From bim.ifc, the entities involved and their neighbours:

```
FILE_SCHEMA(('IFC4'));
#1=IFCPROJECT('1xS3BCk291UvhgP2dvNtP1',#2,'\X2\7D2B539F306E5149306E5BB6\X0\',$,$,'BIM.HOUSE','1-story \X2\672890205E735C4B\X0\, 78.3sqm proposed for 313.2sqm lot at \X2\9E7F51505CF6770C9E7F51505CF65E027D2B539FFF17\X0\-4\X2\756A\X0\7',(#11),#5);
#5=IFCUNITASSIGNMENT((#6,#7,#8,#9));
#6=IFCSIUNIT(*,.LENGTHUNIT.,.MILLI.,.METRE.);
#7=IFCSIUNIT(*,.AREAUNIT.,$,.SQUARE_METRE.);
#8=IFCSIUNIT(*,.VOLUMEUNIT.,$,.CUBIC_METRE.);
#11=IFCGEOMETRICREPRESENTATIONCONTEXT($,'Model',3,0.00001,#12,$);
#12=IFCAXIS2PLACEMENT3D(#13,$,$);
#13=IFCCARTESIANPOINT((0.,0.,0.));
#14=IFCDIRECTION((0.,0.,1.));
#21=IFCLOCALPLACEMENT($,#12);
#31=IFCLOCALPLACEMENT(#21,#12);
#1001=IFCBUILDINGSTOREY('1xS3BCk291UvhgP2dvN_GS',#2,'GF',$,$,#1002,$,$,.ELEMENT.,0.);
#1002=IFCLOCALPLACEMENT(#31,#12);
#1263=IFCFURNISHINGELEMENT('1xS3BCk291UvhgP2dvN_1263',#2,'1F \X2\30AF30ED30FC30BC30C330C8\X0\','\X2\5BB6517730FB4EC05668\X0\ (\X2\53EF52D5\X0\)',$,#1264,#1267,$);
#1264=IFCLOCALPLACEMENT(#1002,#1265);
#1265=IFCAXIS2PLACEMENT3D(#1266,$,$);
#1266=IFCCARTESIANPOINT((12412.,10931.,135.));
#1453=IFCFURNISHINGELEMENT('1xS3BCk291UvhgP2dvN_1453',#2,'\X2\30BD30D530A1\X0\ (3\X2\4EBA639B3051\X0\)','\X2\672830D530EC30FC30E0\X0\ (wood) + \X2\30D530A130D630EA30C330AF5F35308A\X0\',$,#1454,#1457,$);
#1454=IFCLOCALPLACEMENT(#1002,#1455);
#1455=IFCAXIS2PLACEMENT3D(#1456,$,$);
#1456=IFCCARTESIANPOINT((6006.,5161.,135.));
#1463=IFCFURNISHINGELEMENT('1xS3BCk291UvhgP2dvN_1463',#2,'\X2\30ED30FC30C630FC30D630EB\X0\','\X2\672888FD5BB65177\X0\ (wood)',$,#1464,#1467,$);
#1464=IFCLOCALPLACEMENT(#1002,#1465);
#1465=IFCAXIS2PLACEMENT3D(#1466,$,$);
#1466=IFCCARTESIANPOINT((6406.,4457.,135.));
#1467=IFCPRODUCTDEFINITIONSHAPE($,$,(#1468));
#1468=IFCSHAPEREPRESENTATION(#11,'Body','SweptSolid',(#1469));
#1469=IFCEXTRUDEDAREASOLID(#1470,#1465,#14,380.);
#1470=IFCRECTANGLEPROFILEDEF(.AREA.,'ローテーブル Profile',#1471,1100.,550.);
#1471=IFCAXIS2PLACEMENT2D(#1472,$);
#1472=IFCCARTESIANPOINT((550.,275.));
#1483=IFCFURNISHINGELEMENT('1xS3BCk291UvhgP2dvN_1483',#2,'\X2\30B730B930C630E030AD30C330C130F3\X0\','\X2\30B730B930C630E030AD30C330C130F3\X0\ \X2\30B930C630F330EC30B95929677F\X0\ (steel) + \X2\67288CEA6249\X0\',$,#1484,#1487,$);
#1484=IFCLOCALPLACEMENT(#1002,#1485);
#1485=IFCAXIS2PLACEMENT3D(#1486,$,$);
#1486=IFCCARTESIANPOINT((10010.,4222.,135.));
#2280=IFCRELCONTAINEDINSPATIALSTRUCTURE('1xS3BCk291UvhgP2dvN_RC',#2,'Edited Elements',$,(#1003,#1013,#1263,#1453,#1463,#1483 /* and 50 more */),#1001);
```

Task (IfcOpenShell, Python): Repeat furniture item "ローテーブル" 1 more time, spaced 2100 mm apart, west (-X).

```python
import numpy as np
import ifcopenshell
import ifcopenshell.api.geometry
import ifcopenshell.api.root
import ifcopenshell.util.element
import ifcopenshell.util.placement
import ifcopenshell.util.unit

model = ifcopenshell.open("bim.ifc")
unit_scale = ifcopenshell.util.unit.calculate_unit_scale(model)


def reuse_history(source, copy):
    """copy_class also copies each property set's owner history, people and application; keep the originals."""
    for rel in copy.IsDefinedBy:
        if rel.is_a("IfcRelDefinesByProperties") and (history := rel.RelatingPropertyDefinition.OwnerHistory):
            rel.RelatingPropertyDefinition.OwnerHistory = source.OwnerHistory
            ifcopenshell.util.element.remove_deep2(model, history)


source = model.by_guid("1xS3BCk291UvhgP2dvN_1463")
base = ifcopenshell.util.placement.get_local_placement(source.ObjectPlacement)
step = np.array([-1.0, 0.0, 0.0]) * 2.1 / unit_scale

for i in range(1, 2):
    copy = ifcopenshell.api.root.copy_class(model, product=source)
    copy.Representation = ifcopenshell.util.element.copy_deep(
        model, source.Representation, exclude=["IfcGeometricRepresentationContext", "IfcRepresentationMap"]
    )
    reuse_history(source, copy)
    matrix = base.copy()
    matrix[:3, 3] += i * step
    print("added at", matrix[:3, 3].round(3) + 0.0)
    ifcopenshell.api.geometry.edit_object_placement(model, product=copy, matrix=matrix, is_si=False)

model.write("bim_updated.ifc")
```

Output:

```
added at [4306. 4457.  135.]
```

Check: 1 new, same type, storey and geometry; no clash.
